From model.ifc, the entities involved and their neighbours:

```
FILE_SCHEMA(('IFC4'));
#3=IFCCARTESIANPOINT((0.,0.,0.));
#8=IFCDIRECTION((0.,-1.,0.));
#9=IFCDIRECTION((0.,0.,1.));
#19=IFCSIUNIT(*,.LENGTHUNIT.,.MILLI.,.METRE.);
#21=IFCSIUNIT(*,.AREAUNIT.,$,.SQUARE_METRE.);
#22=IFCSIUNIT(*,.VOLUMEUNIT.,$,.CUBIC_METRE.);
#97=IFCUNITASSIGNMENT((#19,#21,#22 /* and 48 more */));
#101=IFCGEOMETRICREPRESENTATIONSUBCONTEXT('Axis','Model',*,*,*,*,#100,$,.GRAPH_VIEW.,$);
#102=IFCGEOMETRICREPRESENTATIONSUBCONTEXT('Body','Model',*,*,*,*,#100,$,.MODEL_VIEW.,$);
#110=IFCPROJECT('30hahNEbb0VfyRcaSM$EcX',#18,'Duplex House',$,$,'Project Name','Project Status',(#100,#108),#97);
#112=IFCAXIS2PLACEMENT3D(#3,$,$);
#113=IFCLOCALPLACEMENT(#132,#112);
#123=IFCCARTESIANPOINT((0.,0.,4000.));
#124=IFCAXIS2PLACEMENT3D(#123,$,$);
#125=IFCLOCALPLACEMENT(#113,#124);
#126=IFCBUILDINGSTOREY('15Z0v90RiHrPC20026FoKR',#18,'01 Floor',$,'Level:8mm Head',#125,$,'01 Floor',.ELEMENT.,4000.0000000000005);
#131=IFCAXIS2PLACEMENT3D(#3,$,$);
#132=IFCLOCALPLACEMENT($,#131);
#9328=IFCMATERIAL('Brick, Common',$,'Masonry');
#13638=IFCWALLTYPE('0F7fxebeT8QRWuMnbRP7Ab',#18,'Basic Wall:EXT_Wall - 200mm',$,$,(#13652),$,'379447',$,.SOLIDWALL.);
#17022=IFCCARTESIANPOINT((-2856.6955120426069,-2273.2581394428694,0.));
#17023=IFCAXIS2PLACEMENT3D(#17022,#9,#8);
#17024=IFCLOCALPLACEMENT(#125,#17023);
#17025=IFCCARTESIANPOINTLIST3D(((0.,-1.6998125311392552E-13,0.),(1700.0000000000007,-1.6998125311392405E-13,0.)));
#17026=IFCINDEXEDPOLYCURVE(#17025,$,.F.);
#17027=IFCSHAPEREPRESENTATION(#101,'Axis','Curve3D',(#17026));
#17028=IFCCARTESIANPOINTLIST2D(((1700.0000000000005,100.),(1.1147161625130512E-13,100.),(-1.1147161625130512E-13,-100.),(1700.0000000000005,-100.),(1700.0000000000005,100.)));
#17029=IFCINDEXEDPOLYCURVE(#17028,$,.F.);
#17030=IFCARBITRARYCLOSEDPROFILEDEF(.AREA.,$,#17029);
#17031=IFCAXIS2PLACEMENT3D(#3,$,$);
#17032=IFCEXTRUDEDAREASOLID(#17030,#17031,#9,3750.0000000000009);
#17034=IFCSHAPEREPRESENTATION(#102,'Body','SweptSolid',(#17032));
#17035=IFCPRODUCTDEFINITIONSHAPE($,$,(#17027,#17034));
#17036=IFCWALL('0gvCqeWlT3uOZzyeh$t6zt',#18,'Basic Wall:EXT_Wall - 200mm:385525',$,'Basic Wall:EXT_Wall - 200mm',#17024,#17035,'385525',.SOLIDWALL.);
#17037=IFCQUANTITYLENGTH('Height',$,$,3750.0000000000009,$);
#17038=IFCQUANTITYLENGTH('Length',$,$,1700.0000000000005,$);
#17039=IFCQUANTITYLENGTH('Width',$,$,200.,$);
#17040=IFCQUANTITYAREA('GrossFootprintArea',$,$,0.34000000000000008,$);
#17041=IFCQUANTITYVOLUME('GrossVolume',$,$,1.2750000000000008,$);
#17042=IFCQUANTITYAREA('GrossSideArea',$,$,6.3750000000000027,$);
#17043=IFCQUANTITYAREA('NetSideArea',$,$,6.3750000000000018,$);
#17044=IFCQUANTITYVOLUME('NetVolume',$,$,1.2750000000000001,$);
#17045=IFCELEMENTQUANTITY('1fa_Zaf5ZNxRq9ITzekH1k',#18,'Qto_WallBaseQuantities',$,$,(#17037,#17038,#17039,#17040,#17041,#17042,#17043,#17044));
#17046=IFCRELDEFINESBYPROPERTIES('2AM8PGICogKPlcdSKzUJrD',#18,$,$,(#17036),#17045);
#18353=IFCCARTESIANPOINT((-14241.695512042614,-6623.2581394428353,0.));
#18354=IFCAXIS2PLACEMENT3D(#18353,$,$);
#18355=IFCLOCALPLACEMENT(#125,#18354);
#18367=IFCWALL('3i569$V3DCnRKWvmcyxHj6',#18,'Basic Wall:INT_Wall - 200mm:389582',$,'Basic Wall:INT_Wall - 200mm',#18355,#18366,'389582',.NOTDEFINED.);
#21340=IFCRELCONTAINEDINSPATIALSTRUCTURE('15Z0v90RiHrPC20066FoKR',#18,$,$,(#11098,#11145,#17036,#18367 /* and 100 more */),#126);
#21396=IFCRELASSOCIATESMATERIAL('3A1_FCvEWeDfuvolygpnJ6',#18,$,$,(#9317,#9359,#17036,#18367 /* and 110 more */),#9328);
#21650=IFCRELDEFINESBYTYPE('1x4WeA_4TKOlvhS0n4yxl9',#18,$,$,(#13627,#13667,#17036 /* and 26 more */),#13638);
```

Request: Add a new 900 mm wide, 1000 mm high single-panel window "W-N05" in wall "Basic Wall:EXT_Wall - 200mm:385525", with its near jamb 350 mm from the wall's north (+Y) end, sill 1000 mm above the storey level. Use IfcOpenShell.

```python
import numpy as np
import ifcopenshell
import ifcopenshell.api.feature
import ifcopenshell.api.geometry
import ifcopenshell.api.pset
import ifcopenshell.api.root
import ifcopenshell.api.spatial
import ifcopenshell.geom
import ifcopenshell.util.element
import ifcopenshell.util.placement
import ifcopenshell.util.representation
import ifcopenshell.util.shape
import ifcopenshell.util.unit

model = ifcopenshell.open("model.ifc")
unit_scale = ifcopenshell.util.unit.calculate_unit_scale(model)
area_scale = ifcopenshell.util.unit.calculate_unit_scale(model, "AREAUNIT")
volume_scale = ifcopenshell.util.unit.calculate_unit_scale(model, "VOLUMEUNIT")
settings = ifcopenshell.geom.settings()


def volume(element):
    """Net volume in cubic metres, openings subtracted."""
    shape = ifcopenshell.geom.create_shape(settings, element)
    return ifcopenshell.util.shape.get_volume(shape.geometry)


wall = model.by_id(17036)
storey = ifcopenshell.util.element.get_container(wall, ifc_class="IfcBuildingStorey")
context = ifcopenshell.util.representation.get_context(model, "Model", "Body", "MODEL_VIEW")
before = volume(wall)

width, height, from_end, sill = 0.9, 1, 0.35, 1  # metres

# The wall runs along its own X axis, and the end named is its -X end.
wall_shape = ifcopenshell.geom.create_shape(settings, wall)
x, y, z = ifcopenshell.util.shape.get_vertices(wall_shape.geometry).T
start = x.min() + from_end
face, thickness = float(y.min()), float(y.max() - y.min())
wall_matrix = ifcopenshell.util.placement.get_local_placement(wall.ObjectPlacement)
level = ifcopenshell.util.placement.get_local_placement(storey.ObjectPlacement)[2, 3]


def in_wall(x, y):
    """Placement at x, y metres in the wall's axes, at sill height."""
    matrix = wall_matrix.copy()
    matrix[:, 3] = wall_matrix @ np.array([x / unit_scale, y / unit_scale, 0.0, 1.0])
    matrix[2, 3] = level + sill / unit_scale
    return matrix


# Opening: a box that overshoots both wall faces by 50 mm.
opening = ifcopenshell.api.root.create_entity(model, ifc_class="IfcOpeningElement", predefined_type="OPENING")
box = ifcopenshell.api.geometry.add_wall_representation(
    model, context=context, length=width, height=height, thickness=thickness + 0.1
)
ifcopenshell.api.geometry.assign_representation(model, product=opening, representation=box)
ifcopenshell.api.geometry.edit_object_placement(model, product=opening, matrix=in_wall(start, face - 0.05), is_si=False)
ifcopenshell.api.feature.add_feature(model, feature=opening, element=wall)

window = ifcopenshell.api.root.create_entity(model, ifc_class="IfcWindow", name="W-N05", predefined_type="WINDOW")
window.OverallWidth, window.OverallHeight = width / unit_scale, height / unit_scale
window.PartitioningType = "SINGLE_PANEL"
body = ifcopenshell.api.geometry.add_window_representation(
    model,
    context=context,
    overall_width=window.OverallWidth,
    overall_height=window.OverallHeight,
    partition_type="SINGLE_PANEL",
)
ifcopenshell.api.geometry.assign_representation(model, product=window, representation=body)
ifcopenshell.api.spatial.assign_container(model, products=[window], relating_structure=storey)
ifcopenshell.api.feature.add_filling(model, opening=opening, element=window)

# Centre the window in the wall's thickness.
ifcopenshell.api.geometry.edit_object_placement(model, product=window, matrix=in_wall(start, face), is_si=False)
window_shape = ifcopenshell.geom.create_shape(settings, window)
depth = ifcopenshell.util.shape.get_vertices(window_shape.geometry)[:, 1]
offset = face + thickness / 2 - (depth.min() + depth.max()) / 2
ifcopenshell.api.geometry.edit_object_placement(model, product=window, matrix=in_wall(start, offset), is_si=False)

after = volume(wall)

# Update the wall's stored quantities.
qto = model.by_id(ifcopenshell.util.element.get_pset(wall, "Qto_WallBaseQuantities", should_inherit=False)["id"])
ifcopenshell.api.pset.edit_qto(model, qto=qto, properties={
    "NetSideArea": after / thickness / area_scale,
    "NetVolume": after / volume_scale,
})

print(f"wall volume {before:.3f} -> {after:.3f} m3")

model.write("model_v2.ifc")
```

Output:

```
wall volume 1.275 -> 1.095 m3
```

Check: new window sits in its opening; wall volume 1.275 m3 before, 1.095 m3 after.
